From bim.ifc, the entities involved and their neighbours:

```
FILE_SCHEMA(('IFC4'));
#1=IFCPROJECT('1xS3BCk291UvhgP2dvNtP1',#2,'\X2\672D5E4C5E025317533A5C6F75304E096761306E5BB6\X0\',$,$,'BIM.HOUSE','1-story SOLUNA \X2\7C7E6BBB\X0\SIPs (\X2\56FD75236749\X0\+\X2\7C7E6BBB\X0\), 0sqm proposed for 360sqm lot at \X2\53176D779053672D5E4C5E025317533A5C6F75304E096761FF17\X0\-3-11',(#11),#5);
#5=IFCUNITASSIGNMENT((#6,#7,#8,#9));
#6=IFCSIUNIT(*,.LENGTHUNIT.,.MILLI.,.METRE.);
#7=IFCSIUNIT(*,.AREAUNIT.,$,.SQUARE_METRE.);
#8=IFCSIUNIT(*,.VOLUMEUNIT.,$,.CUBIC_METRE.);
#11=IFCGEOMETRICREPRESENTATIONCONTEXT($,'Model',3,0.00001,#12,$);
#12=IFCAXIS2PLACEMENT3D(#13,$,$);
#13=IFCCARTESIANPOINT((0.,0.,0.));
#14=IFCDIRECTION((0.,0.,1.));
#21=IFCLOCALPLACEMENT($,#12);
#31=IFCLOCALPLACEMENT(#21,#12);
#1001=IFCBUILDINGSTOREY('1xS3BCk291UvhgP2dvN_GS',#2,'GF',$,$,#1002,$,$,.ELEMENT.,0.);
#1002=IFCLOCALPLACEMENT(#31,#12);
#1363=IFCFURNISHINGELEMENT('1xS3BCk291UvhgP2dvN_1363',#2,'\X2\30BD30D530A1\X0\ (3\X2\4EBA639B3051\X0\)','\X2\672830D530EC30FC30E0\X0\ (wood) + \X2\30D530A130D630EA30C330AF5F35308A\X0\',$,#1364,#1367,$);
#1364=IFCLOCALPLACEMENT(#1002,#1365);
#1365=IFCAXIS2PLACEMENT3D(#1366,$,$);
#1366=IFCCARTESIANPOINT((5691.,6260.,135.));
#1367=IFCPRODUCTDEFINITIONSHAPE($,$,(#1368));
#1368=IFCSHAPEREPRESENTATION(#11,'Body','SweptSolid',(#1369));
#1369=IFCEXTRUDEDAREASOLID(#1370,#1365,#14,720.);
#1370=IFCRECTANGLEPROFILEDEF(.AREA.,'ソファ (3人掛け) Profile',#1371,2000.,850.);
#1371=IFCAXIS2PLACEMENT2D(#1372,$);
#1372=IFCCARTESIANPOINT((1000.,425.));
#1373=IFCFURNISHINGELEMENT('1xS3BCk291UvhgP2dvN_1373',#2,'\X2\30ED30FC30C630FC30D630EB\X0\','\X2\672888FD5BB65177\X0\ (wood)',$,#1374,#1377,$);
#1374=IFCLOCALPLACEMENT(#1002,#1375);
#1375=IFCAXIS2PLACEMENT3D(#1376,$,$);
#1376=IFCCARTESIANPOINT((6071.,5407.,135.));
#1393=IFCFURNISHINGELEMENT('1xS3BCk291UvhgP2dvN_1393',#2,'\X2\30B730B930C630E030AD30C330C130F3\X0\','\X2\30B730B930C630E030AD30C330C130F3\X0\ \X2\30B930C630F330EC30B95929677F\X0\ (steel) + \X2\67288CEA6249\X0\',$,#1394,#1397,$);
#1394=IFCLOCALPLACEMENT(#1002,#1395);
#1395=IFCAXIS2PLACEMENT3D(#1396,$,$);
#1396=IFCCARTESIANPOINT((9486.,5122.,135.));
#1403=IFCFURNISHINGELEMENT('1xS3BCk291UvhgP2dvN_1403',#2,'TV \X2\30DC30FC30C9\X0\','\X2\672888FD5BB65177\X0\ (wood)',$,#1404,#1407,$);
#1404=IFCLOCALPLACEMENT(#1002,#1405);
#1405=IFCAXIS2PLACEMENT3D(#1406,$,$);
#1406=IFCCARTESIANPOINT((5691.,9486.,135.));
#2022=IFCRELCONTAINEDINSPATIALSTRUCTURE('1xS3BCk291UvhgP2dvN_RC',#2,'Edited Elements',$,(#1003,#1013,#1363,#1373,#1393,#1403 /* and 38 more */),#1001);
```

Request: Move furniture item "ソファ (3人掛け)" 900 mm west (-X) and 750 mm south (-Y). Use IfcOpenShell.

```python
import ifcopenshell
import ifcopenshell.api.geometry
import ifcopenshell.util.placement
import ifcopenshell.util.unit

model = ifcopenshell.open("bim.ifc")
unit_scale = ifcopenshell.util.unit.calculate_unit_scale(model)

item = model.by_guid("1xS3BCk291UvhgP2dvN_1363")
matrix = ifcopenshell.util.placement.get_local_placement(item.ObjectPlacement)
matrix[0, 3] -= 0.9 / unit_scale
matrix[1, 3] -= 0.75 / unit_scale
ifcopenshell.api.geometry.edit_object_placement(model, product=item, matrix=matrix, is_si=False)

print(ifcopenshell.util.placement.get_local_placement(item.ObjectPlacement).round(3) + 0.0)

model.write("bim-out.ifc")
```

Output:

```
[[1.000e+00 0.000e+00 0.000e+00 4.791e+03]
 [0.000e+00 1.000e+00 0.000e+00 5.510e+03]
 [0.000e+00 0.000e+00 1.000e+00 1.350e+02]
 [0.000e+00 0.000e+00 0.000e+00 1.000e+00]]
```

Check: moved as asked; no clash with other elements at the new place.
